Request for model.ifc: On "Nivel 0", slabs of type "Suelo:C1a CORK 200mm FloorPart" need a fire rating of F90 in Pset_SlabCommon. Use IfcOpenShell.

First a look at what the model holds.

```python
import ifcopenshell
import ifcopenshell.util.element

model = ifcopenshell.open("model.ifc")
print(model.schema)
storey = next(s for s in model.by_type("IfcBuildingStorey") if s.Name == "Nivel 0")
slabs = [e for e in ifcopenshell.util.element.get_decomposition(storey) if e.is_a("IfcSlab")]
seen = {}
for e in slabs:
    element_type = ifcopenshell.util.element.get_type(e)
    key = (element_type.Name if element_type != e and element_type else None, ifcopenshell.util.element.get_pset(e, "Pset_SlabCommon", "FireRating"))
    seen[key] = seen.get(key, 0) + 1
for (name, value), count in sorted(seen.items(), key=str):
    print(count, "x", name, "|", value)
```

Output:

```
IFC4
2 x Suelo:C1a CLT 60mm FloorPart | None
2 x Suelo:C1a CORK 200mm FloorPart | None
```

```python
import ifcopenshell
import ifcopenshell.api.pset
import ifcopenshell.util.element

model = ifcopenshell.open("model.ifc")

storey = next(s for s in model.by_type("IfcBuildingStorey") if s.Name == "Nivel 0")
slabs = [e for e in ifcopenshell.util.element.get_decomposition(storey) if e.is_a("IfcSlab")]

count = 0
for e in slabs:
    element_type = ifcopenshell.util.element.get_type(e)
    if element_type in (None, e) or element_type.Name != "Suelo:C1a CORK 200mm FloorPart":
        continue
    # add_pset returns the element's existing set when there is one.
    pset = ifcopenshell.api.pset.add_pset(model, product=e, name="Pset_SlabCommon")
    ifcopenshell.api.pset.edit_pset(model, pset=pset, properties={"FireRating": "F90"})
    count += 1

print(count, "slabs updated")

model.write("model_rev.ifc")
```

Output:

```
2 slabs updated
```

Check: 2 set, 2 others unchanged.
